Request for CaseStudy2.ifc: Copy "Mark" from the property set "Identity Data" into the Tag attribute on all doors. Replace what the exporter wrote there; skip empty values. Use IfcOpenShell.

First a look at what the model holds.

```python
import ifcopenshell
import ifcopenshell.util.element

model = ifcopenshell.open("CaseStudy2.ifc")
print(model.schema)
doors = model.by_type("IfcDoor")
print(len(doors), "doors")
for e in doors[:8]:
    source = ifcopenshell.util.element.get_pset(e, "Identity Data", "Mark")
    target = e.Tag
    print(e.id(), repr(source), repr(target), sep=" | ")
```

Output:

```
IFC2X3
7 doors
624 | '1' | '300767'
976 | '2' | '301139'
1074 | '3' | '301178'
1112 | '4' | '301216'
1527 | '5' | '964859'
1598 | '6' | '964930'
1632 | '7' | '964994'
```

```python
import ifcopenshell
import ifcopenshell.util.element

model = ifcopenshell.open("CaseStudy2.ifc")

count = 0
for e in model.by_type("IfcDoor"):
    value = ifcopenshell.util.element.get_pset(e, "Identity Data", "Mark")
    current = e.Tag
    if not value or not value.strip() or current == value:
        continue
    e.Tag = value
    count += 1

print(count, "doors updated")

model.write("CaseStudy2-out.ifc")
```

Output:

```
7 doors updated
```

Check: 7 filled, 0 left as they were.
